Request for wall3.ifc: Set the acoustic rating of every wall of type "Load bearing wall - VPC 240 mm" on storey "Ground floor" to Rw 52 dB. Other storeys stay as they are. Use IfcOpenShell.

First a look at what the model holds.

```python
import ifcopenshell
import ifcopenshell.util.element

model = ifcopenshell.open("wall3.ifc")
print(model.schema)
storey = next(s for s in model.by_type("IfcBuildingStorey") if s.Name == "Ground floor")
walls = [e for e in ifcopenshell.util.element.get_decomposition(storey) if e.is_a("IfcWall")]
seen = {}
for e in walls:
    element_type = ifcopenshell.util.element.get_type(e)
    key = (element_type.Name if element_type != e and element_type else None, ifcopenshell.util.element.get_pset(e, "Pset_WallCommon", "AcousticRating"))
    seen[key] = seen.get(key, 0) + 1
for (name, value), count in sorted(seen.items(), key=str):
    print(count, "x", name, "|", value)
```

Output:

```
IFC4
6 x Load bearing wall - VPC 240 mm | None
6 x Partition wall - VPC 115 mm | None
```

```python
import ifcopenshell
import ifcopenshell.api.pset
import ifcopenshell.util.element

model = ifcopenshell.open("wall3.ifc")

storey = next(s for s in model.by_type("IfcBuildingStorey") if s.Name == "Ground floor")
walls = [e for e in ifcopenshell.util.element.get_decomposition(storey) if e.is_a("IfcWall")]

count = 0
for e in walls:
    element_type = ifcopenshell.util.element.get_type(e)
    if element_type in (None, e) or element_type.Name != "Load bearing wall - VPC 240 mm":
        continue
    # add_pset returns the element's existing set when there is one.
    pset = ifcopenshell.api.pset.add_pset(model, product=e, name="Pset_WallCommon")
    ifcopenshell.api.pset.edit_pset(model, pset=pset, properties={"AcousticRating": "Rw 52 dB"})
    count += 1

print(count, "walls updated")

model.write("wall3_edited.ifc")
```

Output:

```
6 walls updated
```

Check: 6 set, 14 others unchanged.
